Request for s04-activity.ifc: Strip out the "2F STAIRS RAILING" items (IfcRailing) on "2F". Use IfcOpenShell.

First a look at what the model holds.

```python
import ifcopenshell
import ifcopenshell.util.element

model = ifcopenshell.open("s04-activity.ifc")
print(model.schema)
storey = next(s for s in model.by_type("IfcBuildingStorey") if s.Name == "2F")
railings = [e for e in ifcopenshell.util.element.get_decomposition(storey) if e.is_a("IfcRailing")]
seen = {}
for e in railings:
    element_type = ifcopenshell.util.element.get_type(e)
    name = element_type.Name if element_type not in (None, e) else None
    seen[name] = seen.get(name, 0) + 1
for name, count in sorted(seen.items(), key=str):
    print(count, "x", name)
```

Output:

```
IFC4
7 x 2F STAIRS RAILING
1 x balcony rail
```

```python
import ifcopenshell
import ifcopenshell.api.root
import ifcopenshell.util.element

model = ifcopenshell.open("s04-activity.ifc")

storey = next(s for s in model.by_type("IfcBuildingStorey") if s.Name == "2F")
railings = [e for e in ifcopenshell.util.element.get_decomposition(storey) if e.is_a("IfcRailing")]
targets = [e for e in railings if (t := ifcopenshell.util.element.get_type(e)) not in (None, e) and t.Name == "2F STAIRS RAILING"]

for e in targets:
    ifcopenshell.api.root.remove_product(model, product=e)
print(len(targets), "removed")

model.write("s04-activity-out.ifc")
```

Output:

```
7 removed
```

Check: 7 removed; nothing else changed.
